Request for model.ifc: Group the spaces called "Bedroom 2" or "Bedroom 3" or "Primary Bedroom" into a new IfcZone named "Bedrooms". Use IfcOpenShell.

First a look at what the model holds.

```python
import ifcopenshell

model = ifcopenshell.open("model.ifc")
print(model.schema)
seen = {}
for space in model.by_type("IfcSpace"):
    seen[space.LongName] = seen.get(space.LongName, 0) + 1
for name, count in sorted(seen.items(), key=str):
    print(count, "x", name)
print("zones:", [z.Name for z in model.by_type("IfcZone")][:20])
```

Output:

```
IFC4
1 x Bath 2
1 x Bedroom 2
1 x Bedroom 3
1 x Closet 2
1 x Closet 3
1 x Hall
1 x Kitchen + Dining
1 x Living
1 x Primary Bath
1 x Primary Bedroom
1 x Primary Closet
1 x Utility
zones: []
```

```python
import ifcopenshell
import ifcopenshell.api.group
import ifcopenshell.api.root

model = ifcopenshell.open("model.ifc")

names = {"Bedroom 2", "Bedroom 3", "Primary Bedroom"}
spaces = [s for s in model.by_type("IfcSpace") if s.LongName in names]

zone = ifcopenshell.api.root.create_entity(model, ifc_class="IfcZone", name="Bedrooms")
ifcopenshell.api.group.assign_group(model, products=spaces, group=zone)
print(len(spaces), "spaces in", zone.Name)

model.write("model_v2.ifc")
```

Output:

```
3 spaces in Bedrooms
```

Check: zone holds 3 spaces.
